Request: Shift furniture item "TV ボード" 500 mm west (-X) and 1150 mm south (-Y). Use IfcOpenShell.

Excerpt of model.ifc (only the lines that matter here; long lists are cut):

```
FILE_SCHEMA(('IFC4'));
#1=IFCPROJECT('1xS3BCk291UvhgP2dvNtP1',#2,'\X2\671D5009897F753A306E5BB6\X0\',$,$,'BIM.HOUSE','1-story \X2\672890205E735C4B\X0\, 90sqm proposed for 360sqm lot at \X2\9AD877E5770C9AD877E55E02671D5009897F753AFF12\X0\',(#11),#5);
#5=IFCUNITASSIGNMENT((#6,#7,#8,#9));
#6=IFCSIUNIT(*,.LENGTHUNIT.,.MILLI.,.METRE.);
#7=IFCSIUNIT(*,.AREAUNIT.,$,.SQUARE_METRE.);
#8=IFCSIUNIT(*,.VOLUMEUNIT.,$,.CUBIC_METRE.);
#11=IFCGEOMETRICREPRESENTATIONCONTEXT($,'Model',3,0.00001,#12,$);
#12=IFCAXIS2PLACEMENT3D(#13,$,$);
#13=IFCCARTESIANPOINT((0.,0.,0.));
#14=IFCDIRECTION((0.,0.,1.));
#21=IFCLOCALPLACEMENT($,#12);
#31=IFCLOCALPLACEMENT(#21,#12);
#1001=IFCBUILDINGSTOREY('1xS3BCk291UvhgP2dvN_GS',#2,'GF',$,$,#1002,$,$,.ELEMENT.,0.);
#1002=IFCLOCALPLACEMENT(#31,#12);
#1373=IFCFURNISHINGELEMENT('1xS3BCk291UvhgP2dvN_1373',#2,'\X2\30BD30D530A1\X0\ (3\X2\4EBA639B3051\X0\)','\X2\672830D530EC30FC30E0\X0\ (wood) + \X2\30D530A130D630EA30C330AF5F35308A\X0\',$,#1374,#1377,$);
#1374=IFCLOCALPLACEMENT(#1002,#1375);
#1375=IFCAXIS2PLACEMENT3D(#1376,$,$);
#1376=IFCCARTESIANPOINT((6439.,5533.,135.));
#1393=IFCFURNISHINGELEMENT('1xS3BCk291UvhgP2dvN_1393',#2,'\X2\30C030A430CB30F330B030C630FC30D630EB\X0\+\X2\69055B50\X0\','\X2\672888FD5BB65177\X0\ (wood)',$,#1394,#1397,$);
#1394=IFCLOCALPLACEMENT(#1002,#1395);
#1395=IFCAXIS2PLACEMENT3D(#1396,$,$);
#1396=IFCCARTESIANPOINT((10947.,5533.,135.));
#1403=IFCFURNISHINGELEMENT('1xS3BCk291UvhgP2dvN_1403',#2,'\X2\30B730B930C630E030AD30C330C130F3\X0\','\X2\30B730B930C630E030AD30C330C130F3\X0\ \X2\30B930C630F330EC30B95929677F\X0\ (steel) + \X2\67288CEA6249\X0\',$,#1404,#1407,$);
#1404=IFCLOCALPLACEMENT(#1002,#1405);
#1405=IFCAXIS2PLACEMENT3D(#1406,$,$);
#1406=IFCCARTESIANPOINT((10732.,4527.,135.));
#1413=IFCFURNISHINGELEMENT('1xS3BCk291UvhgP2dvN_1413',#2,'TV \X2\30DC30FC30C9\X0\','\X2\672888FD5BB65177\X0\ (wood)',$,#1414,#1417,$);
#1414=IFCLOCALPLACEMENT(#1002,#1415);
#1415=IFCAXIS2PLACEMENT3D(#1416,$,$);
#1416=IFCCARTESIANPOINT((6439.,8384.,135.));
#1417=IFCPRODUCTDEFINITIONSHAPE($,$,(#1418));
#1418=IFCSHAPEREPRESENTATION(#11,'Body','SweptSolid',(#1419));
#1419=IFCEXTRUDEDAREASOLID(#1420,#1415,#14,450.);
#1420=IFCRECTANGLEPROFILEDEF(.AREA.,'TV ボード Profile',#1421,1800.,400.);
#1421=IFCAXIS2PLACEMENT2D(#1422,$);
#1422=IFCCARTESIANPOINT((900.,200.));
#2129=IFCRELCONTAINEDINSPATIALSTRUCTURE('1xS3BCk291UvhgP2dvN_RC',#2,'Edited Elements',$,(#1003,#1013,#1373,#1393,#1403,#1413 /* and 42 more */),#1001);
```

```python
import ifcopenshell
import ifcopenshell.api.geometry
import ifcopenshell.util.placement
import ifcopenshell.util.unit

model = ifcopenshell.open("model.ifc")
unit_scale = ifcopenshell.util.unit.calculate_unit_scale(model)

item = model.by_guid("1xS3BCk291UvhgP2dvN_1413")
matrix = ifcopenshell.util.placement.get_local_placement(item.ObjectPlacement)
matrix[0, 3] -= 0.5 / unit_scale
matrix[1, 3] -= 1.15 / unit_scale
ifcopenshell.api.geometry.edit_object_placement(model, product=item, matrix=matrix, is_si=False)

print(ifcopenshell.util.placement.get_local_placement(item.ObjectPlacement).round(3) + 0.0)

model.write("model_updated.ifc")
```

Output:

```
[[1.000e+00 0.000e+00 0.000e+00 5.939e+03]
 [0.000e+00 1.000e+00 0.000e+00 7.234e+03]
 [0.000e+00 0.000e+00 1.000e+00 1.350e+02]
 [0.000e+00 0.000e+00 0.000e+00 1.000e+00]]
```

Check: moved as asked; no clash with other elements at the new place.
